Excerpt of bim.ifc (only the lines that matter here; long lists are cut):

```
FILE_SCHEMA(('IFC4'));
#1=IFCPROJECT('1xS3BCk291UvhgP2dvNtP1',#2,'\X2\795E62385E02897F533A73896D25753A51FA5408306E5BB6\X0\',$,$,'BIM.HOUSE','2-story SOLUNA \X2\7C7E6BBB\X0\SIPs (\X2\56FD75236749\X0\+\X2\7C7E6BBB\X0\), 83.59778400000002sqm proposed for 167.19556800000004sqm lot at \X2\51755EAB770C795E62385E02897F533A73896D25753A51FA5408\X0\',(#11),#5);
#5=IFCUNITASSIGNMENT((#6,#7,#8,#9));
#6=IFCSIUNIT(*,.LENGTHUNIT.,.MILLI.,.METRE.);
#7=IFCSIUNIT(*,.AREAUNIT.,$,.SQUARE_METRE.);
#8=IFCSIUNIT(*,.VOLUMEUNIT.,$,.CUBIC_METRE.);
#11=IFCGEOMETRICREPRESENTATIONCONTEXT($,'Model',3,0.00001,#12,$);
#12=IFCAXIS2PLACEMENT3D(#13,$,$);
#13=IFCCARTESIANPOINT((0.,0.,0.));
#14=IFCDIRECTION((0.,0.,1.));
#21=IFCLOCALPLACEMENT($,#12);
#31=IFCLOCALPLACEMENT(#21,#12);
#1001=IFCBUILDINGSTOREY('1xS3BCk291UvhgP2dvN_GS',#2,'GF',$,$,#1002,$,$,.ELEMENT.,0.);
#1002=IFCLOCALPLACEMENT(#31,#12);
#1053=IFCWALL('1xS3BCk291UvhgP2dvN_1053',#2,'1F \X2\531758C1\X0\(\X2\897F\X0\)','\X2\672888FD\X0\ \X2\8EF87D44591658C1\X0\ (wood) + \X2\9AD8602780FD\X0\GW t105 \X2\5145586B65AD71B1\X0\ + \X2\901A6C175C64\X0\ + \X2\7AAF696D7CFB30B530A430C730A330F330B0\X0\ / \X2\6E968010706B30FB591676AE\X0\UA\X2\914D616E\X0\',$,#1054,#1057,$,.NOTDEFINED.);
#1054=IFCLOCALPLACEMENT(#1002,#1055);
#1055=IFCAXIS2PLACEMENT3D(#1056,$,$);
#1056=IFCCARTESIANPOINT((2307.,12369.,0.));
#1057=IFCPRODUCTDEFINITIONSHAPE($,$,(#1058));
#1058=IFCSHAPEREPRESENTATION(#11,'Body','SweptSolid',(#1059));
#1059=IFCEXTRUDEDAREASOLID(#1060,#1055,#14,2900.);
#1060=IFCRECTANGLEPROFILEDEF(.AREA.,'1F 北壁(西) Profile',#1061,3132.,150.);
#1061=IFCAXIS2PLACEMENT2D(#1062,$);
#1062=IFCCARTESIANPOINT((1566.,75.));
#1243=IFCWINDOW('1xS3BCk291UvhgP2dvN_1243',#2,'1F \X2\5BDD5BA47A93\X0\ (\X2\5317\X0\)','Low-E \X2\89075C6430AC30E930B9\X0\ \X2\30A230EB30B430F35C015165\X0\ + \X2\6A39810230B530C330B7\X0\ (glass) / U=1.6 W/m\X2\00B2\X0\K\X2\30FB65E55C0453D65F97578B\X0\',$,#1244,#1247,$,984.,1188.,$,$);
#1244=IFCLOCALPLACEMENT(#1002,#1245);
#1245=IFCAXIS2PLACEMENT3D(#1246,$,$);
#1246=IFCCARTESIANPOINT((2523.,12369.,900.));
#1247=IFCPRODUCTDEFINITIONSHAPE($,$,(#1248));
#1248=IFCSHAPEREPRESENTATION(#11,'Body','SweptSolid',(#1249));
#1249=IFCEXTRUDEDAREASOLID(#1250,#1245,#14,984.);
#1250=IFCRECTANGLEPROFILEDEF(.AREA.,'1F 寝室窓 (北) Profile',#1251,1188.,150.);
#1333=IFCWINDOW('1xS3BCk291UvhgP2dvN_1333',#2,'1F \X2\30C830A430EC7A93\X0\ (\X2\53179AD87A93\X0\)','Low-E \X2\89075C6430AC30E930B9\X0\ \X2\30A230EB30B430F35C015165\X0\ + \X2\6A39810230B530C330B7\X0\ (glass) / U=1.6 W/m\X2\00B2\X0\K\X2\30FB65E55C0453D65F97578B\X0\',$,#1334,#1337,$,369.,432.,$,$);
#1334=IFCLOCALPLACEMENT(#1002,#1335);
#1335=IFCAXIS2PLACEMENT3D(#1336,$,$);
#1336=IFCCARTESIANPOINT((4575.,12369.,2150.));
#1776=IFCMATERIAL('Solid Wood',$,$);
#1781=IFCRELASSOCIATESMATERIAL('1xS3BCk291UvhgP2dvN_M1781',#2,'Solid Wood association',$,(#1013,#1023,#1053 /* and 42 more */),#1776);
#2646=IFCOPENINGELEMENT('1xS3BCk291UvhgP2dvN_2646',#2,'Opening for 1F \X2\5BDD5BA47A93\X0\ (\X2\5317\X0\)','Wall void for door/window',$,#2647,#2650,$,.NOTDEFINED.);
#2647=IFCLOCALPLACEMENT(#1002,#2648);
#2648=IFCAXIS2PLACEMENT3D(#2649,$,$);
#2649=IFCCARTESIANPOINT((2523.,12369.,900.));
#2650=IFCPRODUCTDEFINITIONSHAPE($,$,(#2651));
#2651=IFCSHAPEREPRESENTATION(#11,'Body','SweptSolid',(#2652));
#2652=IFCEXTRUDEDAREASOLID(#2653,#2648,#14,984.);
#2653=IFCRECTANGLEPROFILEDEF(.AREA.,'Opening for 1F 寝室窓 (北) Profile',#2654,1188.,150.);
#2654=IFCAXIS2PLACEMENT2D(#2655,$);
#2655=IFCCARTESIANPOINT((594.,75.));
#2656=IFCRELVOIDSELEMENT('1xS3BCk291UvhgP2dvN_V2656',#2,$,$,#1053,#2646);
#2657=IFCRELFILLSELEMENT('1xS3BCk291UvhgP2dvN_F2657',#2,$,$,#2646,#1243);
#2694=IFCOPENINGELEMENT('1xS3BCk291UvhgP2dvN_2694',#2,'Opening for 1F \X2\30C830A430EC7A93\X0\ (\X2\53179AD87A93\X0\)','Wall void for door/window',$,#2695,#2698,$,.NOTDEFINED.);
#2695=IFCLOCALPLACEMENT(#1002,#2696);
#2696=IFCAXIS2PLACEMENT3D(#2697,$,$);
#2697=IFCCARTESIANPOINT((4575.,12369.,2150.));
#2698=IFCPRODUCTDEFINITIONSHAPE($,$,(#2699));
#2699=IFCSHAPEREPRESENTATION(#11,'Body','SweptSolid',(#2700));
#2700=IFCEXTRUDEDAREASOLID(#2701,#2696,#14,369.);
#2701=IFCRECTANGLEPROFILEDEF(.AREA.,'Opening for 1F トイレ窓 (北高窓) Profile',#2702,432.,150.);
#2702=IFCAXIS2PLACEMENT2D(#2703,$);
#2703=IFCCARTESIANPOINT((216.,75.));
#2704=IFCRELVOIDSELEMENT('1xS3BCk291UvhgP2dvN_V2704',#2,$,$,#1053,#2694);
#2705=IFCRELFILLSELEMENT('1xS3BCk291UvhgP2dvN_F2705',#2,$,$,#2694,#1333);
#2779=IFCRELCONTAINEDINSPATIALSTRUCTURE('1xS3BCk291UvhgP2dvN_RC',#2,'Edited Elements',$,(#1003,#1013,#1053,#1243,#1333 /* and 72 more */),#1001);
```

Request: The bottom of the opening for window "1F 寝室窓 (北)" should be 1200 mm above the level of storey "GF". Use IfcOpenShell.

```python
import numpy as np
import ifcopenshell
import ifcopenshell.api.geometry
import ifcopenshell.geom
import ifcopenshell.util.element
import ifcopenshell.util.placement
import ifcopenshell.util.shape
import ifcopenshell.util.unit

model = ifcopenshell.open("bim.ifc")
unit_scale = ifcopenshell.util.unit.calculate_unit_scale(model)

window = model.by_id(1243)
opening = window.FillsVoids[0].RelatingOpeningElement
storey = ifcopenshell.util.element.get_container(window, ifc_class="IfcBuildingStorey")
level = ifcopenshell.util.placement.get_local_placement(storey.ObjectPlacement)[2, 3]

# The opening's origin need not be at the sill, so measure its lowest point.
shape = ifcopenshell.geom.create_shape(ifcopenshell.geom.settings(), opening)
bottom = ifcopenshell.util.shape.get_shape_bottom_elevation(shape, shape.geometry) / unit_scale
dz = level + 1.2 / unit_scale - bottom

shift = np.array([0.0, 0.0, dz])
# The window is not placed relative to its opening, so move both.
for product in (opening, window):
    matrix = ifcopenshell.util.placement.get_local_placement(product.ObjectPlacement)
    matrix[:3, 3] += shift
    ifcopenshell.api.geometry.edit_object_placement(model, product=product, matrix=matrix, is_si=False)

print(f"moved by {dz * unit_scale:+.3f} m")

model.write("bim_v2.ifc")
```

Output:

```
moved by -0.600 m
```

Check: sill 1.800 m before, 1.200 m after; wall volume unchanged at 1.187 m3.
